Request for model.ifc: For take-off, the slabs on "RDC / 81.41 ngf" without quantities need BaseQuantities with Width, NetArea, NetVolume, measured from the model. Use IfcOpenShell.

First a look at what the model holds.

```python
import ifcopenshell
import ifcopenshell.util.element
import ifcopenshell.util.unit

model = ifcopenshell.open("model.ifc")
print(model.schema)
for unit_type in ("LENGTHUNIT", "AREAUNIT", "VOLUMEUNIT"):
    print(unit_type, ifcopenshell.util.unit.calculate_unit_scale(model, unit_type))
storey = next(s for s in model.by_type("IfcBuildingStorey") if s.Name == "RDC / 81.41 ngf")
slabs = [e for e in ifcopenshell.util.element.get_decomposition(storey) if e.is_a("IfcSlab")]
for e in sorted(slabs, key=lambda e: e.id()):
    print(e.id(), e.is_a(), e.Name, list(ifcopenshell.util.element.get_psets(e, qtos_only=True)), sep=" | ")
```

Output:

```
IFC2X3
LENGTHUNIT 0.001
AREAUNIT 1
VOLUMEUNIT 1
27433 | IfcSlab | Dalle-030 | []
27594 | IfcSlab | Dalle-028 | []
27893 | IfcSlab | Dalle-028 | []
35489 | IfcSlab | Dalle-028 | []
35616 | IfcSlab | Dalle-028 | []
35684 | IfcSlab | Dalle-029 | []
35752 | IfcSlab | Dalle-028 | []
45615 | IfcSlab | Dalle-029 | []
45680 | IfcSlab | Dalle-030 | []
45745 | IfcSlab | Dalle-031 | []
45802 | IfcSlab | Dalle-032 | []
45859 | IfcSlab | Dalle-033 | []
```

```python
import ifcopenshell
import ifcopenshell.api.pset
import ifcopenshell.geom
import ifcopenshell.util.element
import ifcopenshell.util.shape
import ifcopenshell.util.unit

model = ifcopenshell.open("model.ifc")
unit_scale = ifcopenshell.util.unit.calculate_unit_scale(model)
area_scale = ifcopenshell.util.unit.calculate_unit_scale(model, "AREAUNIT")
volume_scale = ifcopenshell.util.unit.calculate_unit_scale(model, "VOLUMEUNIT")
settings = ifcopenshell.geom.settings()

storey = next(s for s in model.by_type("IfcBuildingStorey") if s.Name == "RDC / 81.41 ngf")
slabs = [e for e in ifcopenshell.util.element.get_decomposition(storey) if e.is_a("IfcSlab")]

for e in sorted(slabs, key=lambda e: e.id()):
    if ifcopenshell.util.element.get_psets(e, qtos_only=True, should_inherit=False):
        continue
    # Geometry comes back in metres, in the element's own axes.
    shape = ifcopenshell.geom.create_shape(settings, e)
    values = {
        "Width": ifcopenshell.util.shape.get_z(shape.geometry) / unit_scale,
        "NetArea": ifcopenshell.util.shape.get_footprint_area(shape.geometry) / area_scale,
        "NetVolume": ifcopenshell.util.shape.get_volume(shape.geometry) / volume_scale,
    }
    qto = ifcopenshell.api.pset.add_qto(model, product=e, name="BaseQuantities")
    ifcopenshell.api.pset.edit_qto(model, qto=qto, properties=values)
    print(e.id(), {k: round(v, 3) for k, v in values.items()})

model.write("model_v2.ifc")
```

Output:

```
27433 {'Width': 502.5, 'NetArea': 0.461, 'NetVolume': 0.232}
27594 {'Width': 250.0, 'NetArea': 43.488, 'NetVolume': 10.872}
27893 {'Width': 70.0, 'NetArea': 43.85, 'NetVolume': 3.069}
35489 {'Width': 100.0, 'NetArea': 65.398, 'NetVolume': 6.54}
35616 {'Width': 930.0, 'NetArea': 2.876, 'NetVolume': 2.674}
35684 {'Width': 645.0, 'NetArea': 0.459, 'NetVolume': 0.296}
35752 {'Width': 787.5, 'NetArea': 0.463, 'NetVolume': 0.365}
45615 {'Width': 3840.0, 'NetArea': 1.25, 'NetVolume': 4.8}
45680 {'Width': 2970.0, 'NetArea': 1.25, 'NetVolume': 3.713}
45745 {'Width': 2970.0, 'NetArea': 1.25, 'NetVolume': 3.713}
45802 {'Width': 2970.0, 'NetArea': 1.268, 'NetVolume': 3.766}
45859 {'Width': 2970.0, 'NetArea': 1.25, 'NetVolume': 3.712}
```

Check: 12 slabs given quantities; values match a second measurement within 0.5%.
